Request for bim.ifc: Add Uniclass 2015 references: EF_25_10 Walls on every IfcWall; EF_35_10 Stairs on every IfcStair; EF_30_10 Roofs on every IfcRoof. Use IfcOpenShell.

First a look at what the model holds.

```python
import ifcopenshell

model = ifcopenshell.open("bim.ifc")
print(model.schema)
print("classifications:", [c.Name for c in model.by_type("IfcClassification")])
for ifc_class in ("IfcDoor", "IfcRoof", "IfcStair", "IfcWall", "IfcWindow"):
    print(ifc_class, len(model.by_type(ifc_class)))
```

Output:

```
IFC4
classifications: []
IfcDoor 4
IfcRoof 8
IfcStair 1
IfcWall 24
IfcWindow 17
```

```python
import ifcopenshell
import ifcopenshell.api.classification

model = ifcopenshell.open("bim.ifc")

system = ifcopenshell.api.classification.add_classification(model, classification="Uniclass 2015")

codes = {
    "IfcWall": ("EF_25_10", "Walls"),
    "IfcStair": ("EF_35_10", "Stairs"),
    "IfcRoof": ("EF_30_10", "Roofs"),
}
for ifc_class, (code, name) in codes.items():
    products = model.by_type(ifc_class)
    ifcopenshell.api.classification.add_reference(
        model, products=products, classification=system, identification=code, name=name
    )
    print(code, len(products))

model.write("bim_v2.ifc")
```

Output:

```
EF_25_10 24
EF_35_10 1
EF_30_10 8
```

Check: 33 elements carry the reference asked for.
